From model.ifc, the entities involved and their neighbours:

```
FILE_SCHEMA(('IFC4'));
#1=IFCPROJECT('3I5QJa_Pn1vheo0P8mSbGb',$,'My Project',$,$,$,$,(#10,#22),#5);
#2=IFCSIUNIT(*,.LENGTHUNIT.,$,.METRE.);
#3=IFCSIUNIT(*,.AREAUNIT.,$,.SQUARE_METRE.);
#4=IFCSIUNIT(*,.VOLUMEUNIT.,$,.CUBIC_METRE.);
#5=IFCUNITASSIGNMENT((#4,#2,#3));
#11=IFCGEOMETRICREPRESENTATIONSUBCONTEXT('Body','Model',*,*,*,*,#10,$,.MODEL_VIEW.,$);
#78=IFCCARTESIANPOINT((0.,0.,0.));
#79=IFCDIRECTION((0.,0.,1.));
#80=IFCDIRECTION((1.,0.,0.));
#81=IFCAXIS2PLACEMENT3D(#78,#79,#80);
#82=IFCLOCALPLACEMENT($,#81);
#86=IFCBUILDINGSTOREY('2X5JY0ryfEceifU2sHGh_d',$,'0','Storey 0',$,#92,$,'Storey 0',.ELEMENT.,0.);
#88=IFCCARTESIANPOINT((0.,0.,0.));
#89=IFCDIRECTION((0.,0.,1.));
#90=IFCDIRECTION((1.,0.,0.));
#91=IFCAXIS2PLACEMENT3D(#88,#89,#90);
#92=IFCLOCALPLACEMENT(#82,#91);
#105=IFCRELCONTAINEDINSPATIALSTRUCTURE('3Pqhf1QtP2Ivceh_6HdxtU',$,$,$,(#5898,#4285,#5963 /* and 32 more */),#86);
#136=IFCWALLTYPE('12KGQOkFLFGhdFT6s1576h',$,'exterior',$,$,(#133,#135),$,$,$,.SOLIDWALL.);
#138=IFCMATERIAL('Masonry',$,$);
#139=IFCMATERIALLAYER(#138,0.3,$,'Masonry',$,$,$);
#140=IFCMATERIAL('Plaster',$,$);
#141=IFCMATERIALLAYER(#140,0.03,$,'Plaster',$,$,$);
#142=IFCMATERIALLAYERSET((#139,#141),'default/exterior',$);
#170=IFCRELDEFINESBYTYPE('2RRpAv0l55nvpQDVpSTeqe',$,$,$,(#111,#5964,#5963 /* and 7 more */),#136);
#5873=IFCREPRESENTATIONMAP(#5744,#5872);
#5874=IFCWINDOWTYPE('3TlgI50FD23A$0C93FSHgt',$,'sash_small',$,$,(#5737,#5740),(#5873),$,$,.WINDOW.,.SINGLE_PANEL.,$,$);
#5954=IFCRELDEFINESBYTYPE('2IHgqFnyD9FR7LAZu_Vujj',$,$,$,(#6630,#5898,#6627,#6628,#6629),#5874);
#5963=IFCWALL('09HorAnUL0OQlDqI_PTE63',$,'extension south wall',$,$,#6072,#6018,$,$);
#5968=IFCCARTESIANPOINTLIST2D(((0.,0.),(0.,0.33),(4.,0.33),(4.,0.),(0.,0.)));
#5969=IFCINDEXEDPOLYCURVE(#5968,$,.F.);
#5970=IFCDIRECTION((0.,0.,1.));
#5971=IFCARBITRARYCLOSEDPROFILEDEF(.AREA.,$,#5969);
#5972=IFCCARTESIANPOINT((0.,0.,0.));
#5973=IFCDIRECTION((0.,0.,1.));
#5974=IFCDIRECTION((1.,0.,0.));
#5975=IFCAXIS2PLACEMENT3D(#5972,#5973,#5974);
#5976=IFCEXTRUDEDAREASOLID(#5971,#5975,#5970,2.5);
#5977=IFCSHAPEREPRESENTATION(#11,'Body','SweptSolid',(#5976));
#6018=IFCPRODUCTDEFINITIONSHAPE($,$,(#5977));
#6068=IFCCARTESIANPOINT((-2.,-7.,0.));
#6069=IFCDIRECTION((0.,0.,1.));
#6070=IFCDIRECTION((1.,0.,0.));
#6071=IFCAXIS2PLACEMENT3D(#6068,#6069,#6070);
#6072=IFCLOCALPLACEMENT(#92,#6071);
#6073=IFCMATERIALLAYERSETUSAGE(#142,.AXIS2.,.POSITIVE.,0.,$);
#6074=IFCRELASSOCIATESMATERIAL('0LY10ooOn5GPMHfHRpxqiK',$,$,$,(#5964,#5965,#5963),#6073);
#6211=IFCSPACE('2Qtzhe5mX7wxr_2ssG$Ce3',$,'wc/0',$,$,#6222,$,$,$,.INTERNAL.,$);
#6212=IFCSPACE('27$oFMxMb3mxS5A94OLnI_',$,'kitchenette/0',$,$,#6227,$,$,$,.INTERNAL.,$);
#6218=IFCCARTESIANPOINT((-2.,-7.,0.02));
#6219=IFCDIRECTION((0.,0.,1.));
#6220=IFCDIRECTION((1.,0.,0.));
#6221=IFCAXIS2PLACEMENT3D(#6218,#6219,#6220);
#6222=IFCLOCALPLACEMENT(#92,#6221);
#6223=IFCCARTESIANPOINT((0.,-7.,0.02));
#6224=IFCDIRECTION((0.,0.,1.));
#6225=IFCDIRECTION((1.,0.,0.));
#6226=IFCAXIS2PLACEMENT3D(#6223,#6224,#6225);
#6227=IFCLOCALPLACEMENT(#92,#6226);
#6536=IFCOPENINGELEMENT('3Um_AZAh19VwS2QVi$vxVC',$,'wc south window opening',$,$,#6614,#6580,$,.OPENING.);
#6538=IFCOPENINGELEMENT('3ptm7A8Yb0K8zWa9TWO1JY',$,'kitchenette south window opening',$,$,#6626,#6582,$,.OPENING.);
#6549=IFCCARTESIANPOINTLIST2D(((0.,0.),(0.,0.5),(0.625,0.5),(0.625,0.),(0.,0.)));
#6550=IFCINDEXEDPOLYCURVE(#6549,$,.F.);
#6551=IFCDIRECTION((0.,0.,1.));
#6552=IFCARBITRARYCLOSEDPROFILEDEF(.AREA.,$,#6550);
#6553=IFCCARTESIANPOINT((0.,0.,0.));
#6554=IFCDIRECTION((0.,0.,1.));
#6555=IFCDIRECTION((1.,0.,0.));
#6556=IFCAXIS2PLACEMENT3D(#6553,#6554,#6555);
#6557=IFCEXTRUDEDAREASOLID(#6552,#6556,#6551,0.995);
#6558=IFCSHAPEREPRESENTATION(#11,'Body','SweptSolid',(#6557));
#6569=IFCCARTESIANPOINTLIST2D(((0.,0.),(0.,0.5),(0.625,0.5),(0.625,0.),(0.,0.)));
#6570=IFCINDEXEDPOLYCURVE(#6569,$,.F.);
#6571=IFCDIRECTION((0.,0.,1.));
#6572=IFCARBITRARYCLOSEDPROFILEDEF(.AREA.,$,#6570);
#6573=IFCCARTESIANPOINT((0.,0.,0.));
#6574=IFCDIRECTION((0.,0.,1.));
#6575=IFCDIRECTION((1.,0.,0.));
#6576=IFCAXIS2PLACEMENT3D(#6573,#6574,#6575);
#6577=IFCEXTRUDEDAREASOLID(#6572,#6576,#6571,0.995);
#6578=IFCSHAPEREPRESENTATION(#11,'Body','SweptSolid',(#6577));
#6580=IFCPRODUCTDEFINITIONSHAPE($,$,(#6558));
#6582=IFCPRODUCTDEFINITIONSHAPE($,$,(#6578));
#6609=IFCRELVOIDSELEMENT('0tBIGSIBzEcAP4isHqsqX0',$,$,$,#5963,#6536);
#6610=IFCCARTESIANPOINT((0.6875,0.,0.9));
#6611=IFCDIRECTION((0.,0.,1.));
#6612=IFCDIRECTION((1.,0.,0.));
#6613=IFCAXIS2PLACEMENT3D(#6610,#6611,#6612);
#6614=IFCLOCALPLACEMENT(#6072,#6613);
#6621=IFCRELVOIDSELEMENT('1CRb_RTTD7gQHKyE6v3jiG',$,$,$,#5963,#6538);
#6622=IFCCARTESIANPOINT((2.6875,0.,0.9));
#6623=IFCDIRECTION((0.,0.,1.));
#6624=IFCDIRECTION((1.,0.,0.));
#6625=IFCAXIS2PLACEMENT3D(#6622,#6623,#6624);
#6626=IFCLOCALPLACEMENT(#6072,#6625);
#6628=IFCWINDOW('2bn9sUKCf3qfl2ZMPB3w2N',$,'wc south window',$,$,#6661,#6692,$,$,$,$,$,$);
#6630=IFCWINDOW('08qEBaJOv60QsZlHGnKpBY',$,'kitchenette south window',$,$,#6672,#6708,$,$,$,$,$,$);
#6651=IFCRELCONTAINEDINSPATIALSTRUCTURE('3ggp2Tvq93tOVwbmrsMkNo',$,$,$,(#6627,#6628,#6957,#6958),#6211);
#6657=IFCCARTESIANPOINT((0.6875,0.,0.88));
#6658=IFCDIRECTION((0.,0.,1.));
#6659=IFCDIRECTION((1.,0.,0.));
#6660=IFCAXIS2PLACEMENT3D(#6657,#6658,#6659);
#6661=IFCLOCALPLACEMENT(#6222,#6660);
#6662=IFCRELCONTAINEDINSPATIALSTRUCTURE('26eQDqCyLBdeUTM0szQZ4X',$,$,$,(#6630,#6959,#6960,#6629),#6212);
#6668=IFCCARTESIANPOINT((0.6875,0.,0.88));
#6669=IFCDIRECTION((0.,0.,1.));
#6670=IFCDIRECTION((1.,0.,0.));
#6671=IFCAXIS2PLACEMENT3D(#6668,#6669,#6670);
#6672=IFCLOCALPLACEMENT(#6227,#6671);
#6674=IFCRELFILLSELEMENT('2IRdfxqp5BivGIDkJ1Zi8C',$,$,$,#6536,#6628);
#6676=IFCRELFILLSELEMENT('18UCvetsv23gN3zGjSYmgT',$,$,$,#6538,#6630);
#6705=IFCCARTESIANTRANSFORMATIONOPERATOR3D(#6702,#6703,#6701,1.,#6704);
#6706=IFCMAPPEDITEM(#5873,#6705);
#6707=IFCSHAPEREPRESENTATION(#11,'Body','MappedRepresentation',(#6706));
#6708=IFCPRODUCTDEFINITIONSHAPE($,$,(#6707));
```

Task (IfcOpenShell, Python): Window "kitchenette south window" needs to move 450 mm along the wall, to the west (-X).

```python
import ifcopenshell
import ifcopenshell.api.geometry
import ifcopenshell.util.placement
import ifcopenshell.util.unit

model = ifcopenshell.open("model.ifc")
unit_scale = ifcopenshell.util.unit.calculate_unit_scale(model)

window = model.by_id(6630)
opening = window.FillsVoids[0].RelatingOpeningElement
wall = opening.VoidsElements[0].RelatingBuildingElement

wall_matrix = ifcopenshell.util.placement.get_local_placement(wall.ObjectPlacement)
shift = wall_matrix[:3, 0] * -0.45 / unit_scale
before = ifcopenshell.util.placement.get_local_placement(window.ObjectPlacement)[:3, 3].copy()

# The window is not placed relative to its opening, so move both.
for product in (opening, window):
    matrix = ifcopenshell.util.placement.get_local_placement(product.ObjectPlacement)
    matrix[:3, 3] += shift
    ifcopenshell.api.geometry.edit_object_placement(model, product=product, matrix=matrix, is_si=False)

after = ifcopenshell.util.placement.get_local_placement(window.ObjectPlacement)[:3, 3]
print("window moved by", (after - before).round(3) + 0.0)

model.write("model_v2.ifc")
```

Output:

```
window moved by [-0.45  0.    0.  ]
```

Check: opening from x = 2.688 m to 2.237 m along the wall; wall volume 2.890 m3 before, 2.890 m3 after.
